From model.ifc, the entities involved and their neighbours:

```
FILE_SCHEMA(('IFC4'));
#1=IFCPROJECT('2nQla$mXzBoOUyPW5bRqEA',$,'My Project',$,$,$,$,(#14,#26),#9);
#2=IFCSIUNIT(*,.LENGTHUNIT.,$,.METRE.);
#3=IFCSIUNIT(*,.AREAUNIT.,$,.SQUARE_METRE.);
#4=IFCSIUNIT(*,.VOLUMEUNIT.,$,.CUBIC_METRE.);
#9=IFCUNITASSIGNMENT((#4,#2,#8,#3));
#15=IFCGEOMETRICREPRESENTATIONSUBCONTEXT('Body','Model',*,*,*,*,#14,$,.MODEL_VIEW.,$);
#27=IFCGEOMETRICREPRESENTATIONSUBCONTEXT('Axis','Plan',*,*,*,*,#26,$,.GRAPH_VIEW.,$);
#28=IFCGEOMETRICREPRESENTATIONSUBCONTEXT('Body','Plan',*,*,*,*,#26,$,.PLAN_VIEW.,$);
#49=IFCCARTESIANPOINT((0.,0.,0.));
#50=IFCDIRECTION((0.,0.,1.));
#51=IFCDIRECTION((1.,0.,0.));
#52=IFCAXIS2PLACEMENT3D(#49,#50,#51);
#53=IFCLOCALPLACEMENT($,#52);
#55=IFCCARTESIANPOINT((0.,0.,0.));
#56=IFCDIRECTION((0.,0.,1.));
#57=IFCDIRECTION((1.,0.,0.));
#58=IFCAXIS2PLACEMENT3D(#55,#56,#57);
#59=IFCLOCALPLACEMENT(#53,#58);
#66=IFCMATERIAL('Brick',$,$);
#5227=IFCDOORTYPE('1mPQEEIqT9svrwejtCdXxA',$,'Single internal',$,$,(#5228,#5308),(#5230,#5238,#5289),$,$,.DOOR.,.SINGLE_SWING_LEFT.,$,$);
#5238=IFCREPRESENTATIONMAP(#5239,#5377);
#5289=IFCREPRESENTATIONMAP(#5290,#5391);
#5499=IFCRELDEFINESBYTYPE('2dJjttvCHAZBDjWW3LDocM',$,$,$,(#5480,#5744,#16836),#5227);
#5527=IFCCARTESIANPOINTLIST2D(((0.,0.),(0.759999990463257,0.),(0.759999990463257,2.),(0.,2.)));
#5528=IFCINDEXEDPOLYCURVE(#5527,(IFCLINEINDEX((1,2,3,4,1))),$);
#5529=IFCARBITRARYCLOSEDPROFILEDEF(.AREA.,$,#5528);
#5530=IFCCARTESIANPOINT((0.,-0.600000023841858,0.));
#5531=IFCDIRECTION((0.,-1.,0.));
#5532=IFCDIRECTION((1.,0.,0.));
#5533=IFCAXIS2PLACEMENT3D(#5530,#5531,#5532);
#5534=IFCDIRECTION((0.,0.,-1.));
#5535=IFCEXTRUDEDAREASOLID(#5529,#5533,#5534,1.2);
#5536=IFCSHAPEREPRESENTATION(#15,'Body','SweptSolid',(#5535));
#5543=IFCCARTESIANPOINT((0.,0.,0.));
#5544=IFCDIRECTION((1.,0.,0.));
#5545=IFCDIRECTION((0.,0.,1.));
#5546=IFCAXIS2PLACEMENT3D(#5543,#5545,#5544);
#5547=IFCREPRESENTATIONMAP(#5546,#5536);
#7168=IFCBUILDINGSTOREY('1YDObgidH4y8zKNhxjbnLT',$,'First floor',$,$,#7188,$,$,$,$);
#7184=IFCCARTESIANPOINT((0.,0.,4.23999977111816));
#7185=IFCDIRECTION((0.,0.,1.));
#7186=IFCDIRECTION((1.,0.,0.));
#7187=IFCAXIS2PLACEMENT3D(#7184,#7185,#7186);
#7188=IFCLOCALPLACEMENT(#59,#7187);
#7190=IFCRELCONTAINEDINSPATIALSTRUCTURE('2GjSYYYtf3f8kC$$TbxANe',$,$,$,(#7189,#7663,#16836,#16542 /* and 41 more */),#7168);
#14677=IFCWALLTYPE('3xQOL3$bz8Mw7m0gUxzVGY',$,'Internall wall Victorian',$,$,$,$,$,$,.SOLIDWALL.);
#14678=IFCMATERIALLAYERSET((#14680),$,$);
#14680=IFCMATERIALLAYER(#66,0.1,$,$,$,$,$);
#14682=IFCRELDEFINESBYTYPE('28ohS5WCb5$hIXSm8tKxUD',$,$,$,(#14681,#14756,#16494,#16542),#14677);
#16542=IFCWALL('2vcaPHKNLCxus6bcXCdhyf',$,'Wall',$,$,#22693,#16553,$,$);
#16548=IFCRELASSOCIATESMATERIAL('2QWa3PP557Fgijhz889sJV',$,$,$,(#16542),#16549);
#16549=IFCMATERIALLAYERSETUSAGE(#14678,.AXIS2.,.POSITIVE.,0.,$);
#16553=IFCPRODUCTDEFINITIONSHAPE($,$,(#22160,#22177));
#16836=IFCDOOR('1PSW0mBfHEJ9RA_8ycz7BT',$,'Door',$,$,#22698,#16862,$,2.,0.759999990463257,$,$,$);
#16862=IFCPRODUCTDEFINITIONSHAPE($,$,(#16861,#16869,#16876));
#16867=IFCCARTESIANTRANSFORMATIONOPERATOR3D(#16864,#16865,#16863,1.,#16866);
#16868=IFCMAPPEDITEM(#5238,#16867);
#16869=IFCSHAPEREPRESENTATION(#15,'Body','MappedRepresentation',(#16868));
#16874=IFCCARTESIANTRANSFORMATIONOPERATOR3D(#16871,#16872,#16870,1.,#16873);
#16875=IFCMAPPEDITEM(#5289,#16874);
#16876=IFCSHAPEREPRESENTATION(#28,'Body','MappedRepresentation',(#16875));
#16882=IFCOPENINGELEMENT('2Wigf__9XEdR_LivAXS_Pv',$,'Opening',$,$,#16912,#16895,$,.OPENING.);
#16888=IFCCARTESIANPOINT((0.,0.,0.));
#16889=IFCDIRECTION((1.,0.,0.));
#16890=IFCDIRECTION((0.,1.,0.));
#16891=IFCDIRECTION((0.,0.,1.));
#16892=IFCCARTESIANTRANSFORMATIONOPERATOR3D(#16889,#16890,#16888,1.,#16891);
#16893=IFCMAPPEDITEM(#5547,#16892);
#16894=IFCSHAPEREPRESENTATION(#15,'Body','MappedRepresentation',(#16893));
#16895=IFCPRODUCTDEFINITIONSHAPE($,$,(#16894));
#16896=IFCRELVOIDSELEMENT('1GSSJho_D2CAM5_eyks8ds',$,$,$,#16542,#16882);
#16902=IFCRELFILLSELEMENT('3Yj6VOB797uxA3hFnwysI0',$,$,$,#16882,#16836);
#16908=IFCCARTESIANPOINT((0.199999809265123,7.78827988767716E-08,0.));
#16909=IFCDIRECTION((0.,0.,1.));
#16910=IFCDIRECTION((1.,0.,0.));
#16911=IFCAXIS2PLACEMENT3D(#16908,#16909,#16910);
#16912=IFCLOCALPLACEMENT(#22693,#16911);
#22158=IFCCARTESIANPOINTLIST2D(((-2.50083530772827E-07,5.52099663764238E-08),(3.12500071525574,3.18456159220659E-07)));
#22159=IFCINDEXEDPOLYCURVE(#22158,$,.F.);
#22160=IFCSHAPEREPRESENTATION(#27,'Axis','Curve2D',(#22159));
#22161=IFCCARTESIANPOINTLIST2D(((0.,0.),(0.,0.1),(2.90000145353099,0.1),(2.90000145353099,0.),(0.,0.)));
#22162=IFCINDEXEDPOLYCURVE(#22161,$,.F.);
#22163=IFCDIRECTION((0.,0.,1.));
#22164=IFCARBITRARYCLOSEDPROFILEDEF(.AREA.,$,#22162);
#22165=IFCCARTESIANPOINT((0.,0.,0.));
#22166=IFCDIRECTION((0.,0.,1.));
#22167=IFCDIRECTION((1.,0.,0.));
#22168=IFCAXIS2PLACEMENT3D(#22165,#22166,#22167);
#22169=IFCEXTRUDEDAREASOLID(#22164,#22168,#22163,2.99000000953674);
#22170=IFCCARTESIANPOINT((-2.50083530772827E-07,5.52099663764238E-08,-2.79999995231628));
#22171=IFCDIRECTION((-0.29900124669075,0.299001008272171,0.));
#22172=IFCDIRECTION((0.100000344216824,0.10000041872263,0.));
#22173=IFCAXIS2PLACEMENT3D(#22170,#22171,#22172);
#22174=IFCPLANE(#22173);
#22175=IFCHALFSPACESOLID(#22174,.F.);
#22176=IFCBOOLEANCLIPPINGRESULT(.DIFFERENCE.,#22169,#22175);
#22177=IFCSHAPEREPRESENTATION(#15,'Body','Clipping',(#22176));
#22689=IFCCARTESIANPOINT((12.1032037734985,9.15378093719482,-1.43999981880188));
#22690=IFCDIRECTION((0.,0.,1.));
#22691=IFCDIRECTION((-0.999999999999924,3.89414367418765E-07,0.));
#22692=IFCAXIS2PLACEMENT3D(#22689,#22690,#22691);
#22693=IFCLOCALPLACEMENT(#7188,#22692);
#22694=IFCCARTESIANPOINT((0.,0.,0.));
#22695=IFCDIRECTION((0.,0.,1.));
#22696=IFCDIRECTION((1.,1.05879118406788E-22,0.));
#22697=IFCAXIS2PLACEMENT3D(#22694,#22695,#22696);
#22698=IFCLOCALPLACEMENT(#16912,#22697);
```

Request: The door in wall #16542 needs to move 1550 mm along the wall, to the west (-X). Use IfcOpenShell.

```python
import ifcopenshell
import ifcopenshell.api.geometry
import ifcopenshell.util.placement
import ifcopenshell.util.unit

model = ifcopenshell.open("model.ifc")
unit_scale = ifcopenshell.util.unit.calculate_unit_scale(model)

door = model.by_guid("1PSW0mBfHEJ9RA_8ycz7BT")
opening = door.FillsVoids[0].RelatingOpeningElement
wall = opening.VoidsElements[0].RelatingBuildingElement

wall_matrix = ifcopenshell.util.placement.get_local_placement(wall.ObjectPlacement)
shift = wall_matrix[:3, 0] * 1.55 / unit_scale
before = ifcopenshell.util.placement.get_local_placement(door.ObjectPlacement)[:3, 3].copy()

# The door is placed relative to its opening, so it follows when the opening moves.
matrix = ifcopenshell.util.placement.get_local_placement(opening.ObjectPlacement)
matrix[:3, 3] += shift
ifcopenshell.api.geometry.edit_object_placement(
    model, product=opening, matrix=matrix, is_si=False, should_transform_children=True
)

after = ifcopenshell.util.placement.get_local_placement(door.ObjectPlacement)[:3, 3]
print("door moved by", (after - before).round(3) + 0.0)

model.write("model_updated.ifc")
```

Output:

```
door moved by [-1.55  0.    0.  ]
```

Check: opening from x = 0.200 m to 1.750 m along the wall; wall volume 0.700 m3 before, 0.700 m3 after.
